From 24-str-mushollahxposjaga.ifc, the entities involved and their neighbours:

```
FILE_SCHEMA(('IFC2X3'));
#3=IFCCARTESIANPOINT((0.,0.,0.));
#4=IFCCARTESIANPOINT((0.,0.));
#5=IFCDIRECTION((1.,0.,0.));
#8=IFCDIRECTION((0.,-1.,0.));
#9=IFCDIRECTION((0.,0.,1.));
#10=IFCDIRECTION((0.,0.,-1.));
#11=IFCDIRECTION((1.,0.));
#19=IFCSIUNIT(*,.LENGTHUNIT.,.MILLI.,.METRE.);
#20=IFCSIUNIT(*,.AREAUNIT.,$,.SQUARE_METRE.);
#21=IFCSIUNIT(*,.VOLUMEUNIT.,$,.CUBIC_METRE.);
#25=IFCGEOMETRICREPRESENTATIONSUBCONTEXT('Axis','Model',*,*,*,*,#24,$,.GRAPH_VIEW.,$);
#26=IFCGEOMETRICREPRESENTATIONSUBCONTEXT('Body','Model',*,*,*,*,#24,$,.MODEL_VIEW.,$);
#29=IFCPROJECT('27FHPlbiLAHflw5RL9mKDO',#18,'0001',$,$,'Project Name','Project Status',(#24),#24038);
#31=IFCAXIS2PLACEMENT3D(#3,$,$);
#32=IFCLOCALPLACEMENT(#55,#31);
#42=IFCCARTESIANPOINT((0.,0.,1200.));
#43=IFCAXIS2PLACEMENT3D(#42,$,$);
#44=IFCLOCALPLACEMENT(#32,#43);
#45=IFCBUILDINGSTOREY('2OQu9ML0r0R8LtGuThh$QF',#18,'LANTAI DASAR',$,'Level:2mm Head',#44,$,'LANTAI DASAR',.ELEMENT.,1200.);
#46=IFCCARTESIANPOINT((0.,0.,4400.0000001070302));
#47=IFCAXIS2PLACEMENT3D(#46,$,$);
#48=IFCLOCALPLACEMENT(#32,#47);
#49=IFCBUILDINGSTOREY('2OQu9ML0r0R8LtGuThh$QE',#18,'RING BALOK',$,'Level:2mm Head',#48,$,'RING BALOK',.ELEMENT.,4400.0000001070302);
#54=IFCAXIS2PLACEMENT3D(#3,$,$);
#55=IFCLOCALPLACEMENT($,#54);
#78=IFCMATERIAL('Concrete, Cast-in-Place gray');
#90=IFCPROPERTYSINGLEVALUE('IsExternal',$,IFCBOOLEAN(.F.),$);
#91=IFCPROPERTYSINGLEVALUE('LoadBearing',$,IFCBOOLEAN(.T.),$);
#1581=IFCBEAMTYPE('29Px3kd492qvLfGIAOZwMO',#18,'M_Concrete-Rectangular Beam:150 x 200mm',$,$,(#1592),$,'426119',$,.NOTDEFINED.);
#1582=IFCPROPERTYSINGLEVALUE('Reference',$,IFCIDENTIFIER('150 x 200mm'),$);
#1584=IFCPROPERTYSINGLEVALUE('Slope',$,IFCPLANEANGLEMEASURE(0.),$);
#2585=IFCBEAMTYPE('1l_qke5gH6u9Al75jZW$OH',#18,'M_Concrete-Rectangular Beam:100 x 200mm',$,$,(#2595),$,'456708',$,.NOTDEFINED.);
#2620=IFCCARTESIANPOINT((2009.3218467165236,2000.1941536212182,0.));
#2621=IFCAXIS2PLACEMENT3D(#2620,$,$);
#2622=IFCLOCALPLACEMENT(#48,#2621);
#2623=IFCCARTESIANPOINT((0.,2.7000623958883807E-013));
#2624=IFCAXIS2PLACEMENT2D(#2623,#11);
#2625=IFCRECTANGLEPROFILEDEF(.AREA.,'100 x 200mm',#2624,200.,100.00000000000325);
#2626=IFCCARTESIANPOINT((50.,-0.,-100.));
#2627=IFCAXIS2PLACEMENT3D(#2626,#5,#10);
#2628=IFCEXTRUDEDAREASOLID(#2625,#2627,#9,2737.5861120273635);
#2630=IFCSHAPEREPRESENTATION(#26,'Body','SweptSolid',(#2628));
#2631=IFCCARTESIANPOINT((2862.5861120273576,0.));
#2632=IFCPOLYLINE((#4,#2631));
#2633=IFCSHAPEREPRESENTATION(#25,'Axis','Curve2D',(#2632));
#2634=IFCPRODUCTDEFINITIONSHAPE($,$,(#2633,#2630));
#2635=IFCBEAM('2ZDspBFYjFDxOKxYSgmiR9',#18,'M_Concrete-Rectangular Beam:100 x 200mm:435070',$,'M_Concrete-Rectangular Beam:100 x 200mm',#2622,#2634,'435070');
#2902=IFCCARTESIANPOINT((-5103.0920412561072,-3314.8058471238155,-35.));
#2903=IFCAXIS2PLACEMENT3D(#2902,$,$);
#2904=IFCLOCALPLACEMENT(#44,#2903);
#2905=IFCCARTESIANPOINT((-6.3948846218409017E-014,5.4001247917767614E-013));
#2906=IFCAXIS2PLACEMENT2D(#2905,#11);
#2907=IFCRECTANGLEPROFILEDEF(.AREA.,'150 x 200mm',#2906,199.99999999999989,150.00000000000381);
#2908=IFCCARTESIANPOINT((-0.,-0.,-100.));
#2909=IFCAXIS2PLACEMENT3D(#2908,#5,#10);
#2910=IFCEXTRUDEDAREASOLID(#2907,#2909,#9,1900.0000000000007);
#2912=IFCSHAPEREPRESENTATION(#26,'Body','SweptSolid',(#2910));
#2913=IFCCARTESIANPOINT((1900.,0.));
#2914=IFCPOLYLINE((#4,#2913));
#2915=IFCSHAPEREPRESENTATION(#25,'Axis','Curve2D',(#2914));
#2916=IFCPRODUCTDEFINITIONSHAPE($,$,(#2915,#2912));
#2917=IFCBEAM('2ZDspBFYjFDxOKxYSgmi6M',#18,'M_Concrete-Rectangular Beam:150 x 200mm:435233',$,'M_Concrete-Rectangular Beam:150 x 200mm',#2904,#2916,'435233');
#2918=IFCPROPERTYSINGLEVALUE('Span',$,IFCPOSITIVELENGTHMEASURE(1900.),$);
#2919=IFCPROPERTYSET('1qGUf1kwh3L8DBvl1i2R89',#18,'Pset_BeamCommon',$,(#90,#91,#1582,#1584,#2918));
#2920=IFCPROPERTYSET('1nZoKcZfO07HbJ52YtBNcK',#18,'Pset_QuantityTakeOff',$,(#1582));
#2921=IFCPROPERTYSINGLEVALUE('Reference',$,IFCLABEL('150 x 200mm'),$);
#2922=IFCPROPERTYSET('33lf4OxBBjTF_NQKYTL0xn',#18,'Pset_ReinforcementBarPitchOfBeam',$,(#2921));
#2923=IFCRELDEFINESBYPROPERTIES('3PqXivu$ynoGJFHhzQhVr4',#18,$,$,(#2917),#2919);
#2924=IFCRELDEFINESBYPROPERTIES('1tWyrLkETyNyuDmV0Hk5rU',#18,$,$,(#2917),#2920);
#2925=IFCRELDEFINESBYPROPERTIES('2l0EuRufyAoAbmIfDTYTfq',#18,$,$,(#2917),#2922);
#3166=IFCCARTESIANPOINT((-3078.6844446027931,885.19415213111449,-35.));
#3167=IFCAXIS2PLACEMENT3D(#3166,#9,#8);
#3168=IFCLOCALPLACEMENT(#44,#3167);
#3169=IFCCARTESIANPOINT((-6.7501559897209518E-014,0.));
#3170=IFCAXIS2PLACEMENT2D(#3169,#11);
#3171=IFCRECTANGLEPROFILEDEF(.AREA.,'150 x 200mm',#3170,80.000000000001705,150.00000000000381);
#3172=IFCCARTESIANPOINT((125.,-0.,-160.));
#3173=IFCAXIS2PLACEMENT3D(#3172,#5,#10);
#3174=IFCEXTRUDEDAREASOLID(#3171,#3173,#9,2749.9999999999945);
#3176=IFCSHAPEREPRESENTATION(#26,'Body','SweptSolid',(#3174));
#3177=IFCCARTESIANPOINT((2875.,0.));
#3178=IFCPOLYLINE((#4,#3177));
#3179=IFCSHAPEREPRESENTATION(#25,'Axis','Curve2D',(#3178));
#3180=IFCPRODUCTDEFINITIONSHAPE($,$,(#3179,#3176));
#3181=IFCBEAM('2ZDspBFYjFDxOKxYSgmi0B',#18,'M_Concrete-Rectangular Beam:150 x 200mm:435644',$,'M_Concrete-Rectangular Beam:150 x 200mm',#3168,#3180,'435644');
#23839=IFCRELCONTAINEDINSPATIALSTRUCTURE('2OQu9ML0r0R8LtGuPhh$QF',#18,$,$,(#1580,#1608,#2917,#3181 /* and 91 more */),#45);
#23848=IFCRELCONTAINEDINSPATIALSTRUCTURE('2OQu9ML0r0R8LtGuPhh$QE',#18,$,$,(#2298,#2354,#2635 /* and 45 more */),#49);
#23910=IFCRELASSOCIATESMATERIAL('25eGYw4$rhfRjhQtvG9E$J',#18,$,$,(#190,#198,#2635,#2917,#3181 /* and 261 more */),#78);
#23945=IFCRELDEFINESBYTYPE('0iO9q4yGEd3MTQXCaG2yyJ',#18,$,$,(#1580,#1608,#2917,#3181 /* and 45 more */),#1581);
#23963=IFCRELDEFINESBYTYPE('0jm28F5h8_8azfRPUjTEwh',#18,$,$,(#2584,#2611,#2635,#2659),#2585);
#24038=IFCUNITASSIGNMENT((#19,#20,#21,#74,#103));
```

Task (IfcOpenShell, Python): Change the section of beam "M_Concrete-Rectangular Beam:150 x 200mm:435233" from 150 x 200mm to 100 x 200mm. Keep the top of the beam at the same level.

```python
import ifcopenshell
import ifcopenshell.api.pset
import ifcopenshell.api.type
import ifcopenshell.util.element
import ifcopenshell.util.representation

model = ifcopenshell.open("24-str-mushollahxposjaga.ifc")

member = model.by_id(2917)
source = next(p for p in model.by_type("IfcRectangleProfileDef") if p.ProfileName == "100 x 200mm")

body = ifcopenshell.util.representation.get_representation(member, "Model", "Body")
solid = body.Items[0]
old_profile = solid.SweptArea

# Copy the section's sizes but keep this member's own profile position.
profile = ifcopenshell.util.element.copy(model, source)
# Profiles are centred, so shift by half the change in depth to hold the top.
shift = (old_profile.XDim - profile.XDim) / 2
x, y = old_profile.Position.Location.Coordinates
up = (-1.0, 0.0)  # upwards, in the solid's own plane
location = model.createIfcCartesianPoint((x + up[0] * shift, y + up[1] * shift))
profile.Position = model.createIfcAxis2Placement2D(location, old_profile.Position.RefDirection)
solid.SweptArea = profile
if not model.get_total_inverses(old_profile):
    ifcopenshell.util.element.remove_deep2(model, old_profile)

new_type = model.by_guid("1l_qke5gH6u9Al75jZW$OH")
ifcopenshell.api.type.assign_type(
    model, related_objects=[member], relating_type=new_type, should_map_representations=False
)
member.Name = member.Name.replace("150 x 200mm", "100 x 200mm")
member.ObjectType = "M_Concrete-Rectangular Beam:100 x 200mm"
pset = model.by_id(ifcopenshell.util.element.get_pset(member, "Pset_BeamCommon", should_inherit=False)["id"])
ifcopenshell.api.pset.edit_pset(model, pset=pset, properties={"Reference": "100 x 200mm"})
pset = model.by_id(ifcopenshell.util.element.get_pset(member, "Pset_QuantityTakeOff", should_inherit=False)["id"])
ifcopenshell.api.pset.edit_pset(model, pset=pset, properties={"Reference": "100 x 200mm"})
pset = model.by_id(ifcopenshell.util.element.get_pset(member, "Pset_ReinforcementBarPitchOfBeam", should_inherit=False)["id"])
ifcopenshell.api.pset.edit_pset(model, pset=pset, properties={"Reference": "100 x 200mm"})

print(solid.SweptArea)

model.write("24-str-mushollahxposjaga_edited.ifc")
```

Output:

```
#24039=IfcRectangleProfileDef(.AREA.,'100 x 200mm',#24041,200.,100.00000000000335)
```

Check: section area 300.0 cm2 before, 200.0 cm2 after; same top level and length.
